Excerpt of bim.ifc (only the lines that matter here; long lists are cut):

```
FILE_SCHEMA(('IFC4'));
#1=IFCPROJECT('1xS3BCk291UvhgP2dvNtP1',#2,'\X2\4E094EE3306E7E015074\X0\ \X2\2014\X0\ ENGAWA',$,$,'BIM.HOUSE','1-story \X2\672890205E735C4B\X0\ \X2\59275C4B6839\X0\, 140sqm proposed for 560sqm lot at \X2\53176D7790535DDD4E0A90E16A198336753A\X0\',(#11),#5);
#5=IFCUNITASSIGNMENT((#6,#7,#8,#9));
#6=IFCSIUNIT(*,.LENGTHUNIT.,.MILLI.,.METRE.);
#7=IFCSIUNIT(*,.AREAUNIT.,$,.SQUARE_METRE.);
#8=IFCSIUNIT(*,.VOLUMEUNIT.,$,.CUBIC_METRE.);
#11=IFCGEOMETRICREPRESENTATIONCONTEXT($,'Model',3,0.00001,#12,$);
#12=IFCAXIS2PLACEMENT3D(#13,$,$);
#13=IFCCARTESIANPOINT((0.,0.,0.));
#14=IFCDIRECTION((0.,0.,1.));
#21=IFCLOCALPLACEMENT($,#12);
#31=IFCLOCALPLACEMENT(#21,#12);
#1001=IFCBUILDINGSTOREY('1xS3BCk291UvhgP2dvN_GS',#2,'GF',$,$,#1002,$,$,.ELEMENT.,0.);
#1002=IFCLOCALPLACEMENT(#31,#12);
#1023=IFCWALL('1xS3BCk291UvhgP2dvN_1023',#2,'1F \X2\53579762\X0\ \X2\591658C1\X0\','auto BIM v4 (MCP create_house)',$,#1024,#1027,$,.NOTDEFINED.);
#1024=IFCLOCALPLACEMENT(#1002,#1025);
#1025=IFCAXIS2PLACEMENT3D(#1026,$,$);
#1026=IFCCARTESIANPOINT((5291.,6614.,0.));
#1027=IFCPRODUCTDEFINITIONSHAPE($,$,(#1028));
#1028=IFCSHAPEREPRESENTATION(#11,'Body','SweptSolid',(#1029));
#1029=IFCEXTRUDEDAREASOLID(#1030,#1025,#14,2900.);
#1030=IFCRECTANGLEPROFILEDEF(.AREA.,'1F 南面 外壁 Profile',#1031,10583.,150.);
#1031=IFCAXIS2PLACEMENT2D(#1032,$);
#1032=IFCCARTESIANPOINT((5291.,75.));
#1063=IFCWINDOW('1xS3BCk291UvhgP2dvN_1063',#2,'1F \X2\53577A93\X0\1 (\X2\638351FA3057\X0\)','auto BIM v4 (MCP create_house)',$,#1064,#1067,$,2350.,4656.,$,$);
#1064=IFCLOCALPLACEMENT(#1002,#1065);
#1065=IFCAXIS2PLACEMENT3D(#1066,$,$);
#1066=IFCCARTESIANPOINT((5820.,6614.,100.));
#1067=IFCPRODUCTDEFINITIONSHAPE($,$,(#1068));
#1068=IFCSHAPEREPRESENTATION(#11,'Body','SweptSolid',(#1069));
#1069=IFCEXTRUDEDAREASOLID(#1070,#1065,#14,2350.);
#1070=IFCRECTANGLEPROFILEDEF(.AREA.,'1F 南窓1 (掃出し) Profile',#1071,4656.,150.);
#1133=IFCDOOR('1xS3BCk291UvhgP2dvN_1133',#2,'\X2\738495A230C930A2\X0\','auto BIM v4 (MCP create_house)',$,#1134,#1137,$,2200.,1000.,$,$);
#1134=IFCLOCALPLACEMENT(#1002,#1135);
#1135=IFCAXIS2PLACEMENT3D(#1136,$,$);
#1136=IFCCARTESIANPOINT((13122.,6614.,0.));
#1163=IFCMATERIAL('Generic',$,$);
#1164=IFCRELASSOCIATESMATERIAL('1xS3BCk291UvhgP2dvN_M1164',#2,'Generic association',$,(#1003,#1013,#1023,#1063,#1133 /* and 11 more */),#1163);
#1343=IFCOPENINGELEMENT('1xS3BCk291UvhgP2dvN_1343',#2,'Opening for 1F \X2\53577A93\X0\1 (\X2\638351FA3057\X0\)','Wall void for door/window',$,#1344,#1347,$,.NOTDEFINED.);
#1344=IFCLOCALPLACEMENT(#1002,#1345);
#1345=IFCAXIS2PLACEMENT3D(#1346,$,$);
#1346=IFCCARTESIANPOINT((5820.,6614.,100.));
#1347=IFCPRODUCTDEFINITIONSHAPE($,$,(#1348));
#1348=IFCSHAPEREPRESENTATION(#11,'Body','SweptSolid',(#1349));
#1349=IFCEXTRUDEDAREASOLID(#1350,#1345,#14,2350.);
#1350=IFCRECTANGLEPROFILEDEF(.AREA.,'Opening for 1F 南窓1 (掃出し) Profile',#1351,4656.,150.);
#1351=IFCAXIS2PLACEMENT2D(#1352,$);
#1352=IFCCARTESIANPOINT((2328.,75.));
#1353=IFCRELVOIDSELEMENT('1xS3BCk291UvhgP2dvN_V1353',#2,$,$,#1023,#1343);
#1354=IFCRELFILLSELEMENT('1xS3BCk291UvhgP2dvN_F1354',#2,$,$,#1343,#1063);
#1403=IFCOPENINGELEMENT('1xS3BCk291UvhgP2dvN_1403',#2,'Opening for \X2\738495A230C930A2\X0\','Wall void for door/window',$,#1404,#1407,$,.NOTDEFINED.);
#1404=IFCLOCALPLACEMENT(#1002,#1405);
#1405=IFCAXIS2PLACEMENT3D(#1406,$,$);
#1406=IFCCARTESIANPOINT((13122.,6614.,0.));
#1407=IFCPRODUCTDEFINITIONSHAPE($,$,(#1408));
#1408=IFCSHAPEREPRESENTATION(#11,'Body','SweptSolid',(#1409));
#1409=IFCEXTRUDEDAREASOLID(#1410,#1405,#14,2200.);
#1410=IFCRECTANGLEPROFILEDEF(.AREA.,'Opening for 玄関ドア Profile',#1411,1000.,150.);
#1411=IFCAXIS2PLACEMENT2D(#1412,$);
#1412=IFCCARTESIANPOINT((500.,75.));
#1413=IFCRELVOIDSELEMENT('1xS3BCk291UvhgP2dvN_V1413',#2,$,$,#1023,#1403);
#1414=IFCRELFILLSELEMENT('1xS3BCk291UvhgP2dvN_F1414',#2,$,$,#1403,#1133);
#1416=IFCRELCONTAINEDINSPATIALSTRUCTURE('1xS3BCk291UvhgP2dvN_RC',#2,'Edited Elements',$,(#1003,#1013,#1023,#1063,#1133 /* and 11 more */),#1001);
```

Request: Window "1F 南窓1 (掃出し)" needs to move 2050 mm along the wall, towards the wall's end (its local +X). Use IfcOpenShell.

```python
import ifcopenshell
import ifcopenshell.api.geometry
import ifcopenshell.util.placement
import ifcopenshell.util.unit

model = ifcopenshell.open("bim.ifc")
unit_scale = ifcopenshell.util.unit.calculate_unit_scale(model)

window = model.by_guid("1xS3BCk291UvhgP2dvN_1063")
opening = window.FillsVoids[0].RelatingOpeningElement
wall = opening.VoidsElements[0].RelatingBuildingElement

wall_matrix = ifcopenshell.util.placement.get_local_placement(wall.ObjectPlacement)
shift = wall_matrix[:3, 0] * 2.05 / unit_scale
before = ifcopenshell.util.placement.get_local_placement(window.ObjectPlacement)[:3, 3].copy()

# The window is not placed relative to its opening, so move both.
for product in (opening, window):
    matrix = ifcopenshell.util.placement.get_local_placement(product.ObjectPlacement)
    matrix[:3, 3] += shift
    ifcopenshell.api.geometry.edit_object_placement(model, product=product, matrix=matrix, is_si=False)

after = ifcopenshell.util.placement.get_local_placement(window.ObjectPlacement)[:3, 3]
print("window moved by", (after - before).round(3) + 0.0)

model.write("bim_rev.ifc")
```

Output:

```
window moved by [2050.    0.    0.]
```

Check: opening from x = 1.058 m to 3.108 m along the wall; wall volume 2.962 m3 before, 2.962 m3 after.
